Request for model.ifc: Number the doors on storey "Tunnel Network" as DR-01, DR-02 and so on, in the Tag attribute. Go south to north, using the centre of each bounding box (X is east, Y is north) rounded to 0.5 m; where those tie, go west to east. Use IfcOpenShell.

First a look at what the model holds.

```python
import ifcopenshell
import ifcopenshell.util.element
import ifcopenshell.util.placement

model = ifcopenshell.open("model.ifc")
print(model.schema)
storey = next(s for s in model.by_type("IfcBuildingStorey") if s.Name == "Tunnel Network")
doors = [e for e in ifcopenshell.util.element.get_decomposition(storey) if e.is_a("IfcDoor")]
for e in sorted(doors, key=lambda e: e.id()):
    origin = ifcopenshell.util.placement.get_local_placement(e.ObjectPlacement)[:3, 3]
    print(e.id(), e.Tag, e.Name, origin.round(2) + 0.0, sep=" | ")
```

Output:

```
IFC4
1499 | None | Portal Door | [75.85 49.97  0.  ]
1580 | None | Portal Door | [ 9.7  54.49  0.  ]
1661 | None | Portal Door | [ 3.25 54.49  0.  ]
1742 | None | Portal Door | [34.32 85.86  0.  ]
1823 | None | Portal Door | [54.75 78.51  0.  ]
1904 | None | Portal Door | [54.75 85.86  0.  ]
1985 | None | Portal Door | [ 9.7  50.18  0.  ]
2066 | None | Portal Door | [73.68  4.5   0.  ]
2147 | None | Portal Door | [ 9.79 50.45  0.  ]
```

```python
import ifcopenshell
import ifcopenshell.geom
import ifcopenshell.util.element
import ifcopenshell.util.shape

model = ifcopenshell.open("model.ifc")
settings = ifcopenshell.geom.settings()
settings.set("use-world-coords", True)


def centre(element):
    shape = ifcopenshell.geom.create_shape(settings, element)
    return ifcopenshell.util.shape.get_bbox_centroid(shape.geometry)


storey = next(s for s in model.by_type("IfcBuildingStorey") if s.Name == "Tunnel Network")
doors = [e for e in ifcopenshell.util.element.get_decomposition(storey) if e.is_a("IfcDoor")]

# Insertion points can sit at a corner or the storey origin, so sort by the geometry (in metres).
centres = {e: centre(e) for e in doors}
doors.sort(key=lambda e: (round(centres[e][1] / 0.5), centres[e][0]))

for i, e in enumerate(doors, start=1):
    number = f"DR-{i:02d}"
    e.Tag = number
    print(e.id(), number)

model.write("model_v2.ifc")
```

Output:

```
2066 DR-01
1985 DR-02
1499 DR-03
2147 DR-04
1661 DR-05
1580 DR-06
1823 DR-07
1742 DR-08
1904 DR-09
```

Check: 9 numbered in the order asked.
